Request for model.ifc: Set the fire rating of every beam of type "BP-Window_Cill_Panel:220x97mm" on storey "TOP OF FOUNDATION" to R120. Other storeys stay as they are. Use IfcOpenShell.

First a look at what the model holds.

```python
import ifcopenshell
import ifcopenshell.util.element

model = ifcopenshell.open("model.ifc")
print(model.schema)
storey = next(s for s in model.by_type("IfcBuildingStorey") if s.Name == "TOP OF FOUNDATION")
beams = [e for e in ifcopenshell.util.element.get_decomposition(storey) if e.is_a("IfcBeam")]
seen = {}
for e in beams:
    element_type = ifcopenshell.util.element.get_type(e)
    key = (element_type.Name if element_type != e and element_type else None, ifcopenshell.util.element.get_pset(e, "Pset_BeamCommon", "FireRating"))
    seen[key] = seen.get(key, 0) + 1
for (name, value), count in sorted(seen.items(), key=str):
    print(count, "x", name, "|", value)
```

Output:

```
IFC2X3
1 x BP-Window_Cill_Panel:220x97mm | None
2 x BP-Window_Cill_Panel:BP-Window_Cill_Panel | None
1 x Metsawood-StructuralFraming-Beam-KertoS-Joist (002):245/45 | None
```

```python
import ifcopenshell
import ifcopenshell.api.pset
import ifcopenshell.util.element

model = ifcopenshell.open("model.ifc")

storey = next(s for s in model.by_type("IfcBuildingStorey") if s.Name == "TOP OF FOUNDATION")
beams = [e for e in ifcopenshell.util.element.get_decomposition(storey) if e.is_a("IfcBeam")]

count = 0
for e in beams:
    element_type = ifcopenshell.util.element.get_type(e)
    if element_type in (None, e) or element_type.Name != "BP-Window_Cill_Panel:220x97mm":
        continue
    # add_pset returns the element's existing set when there is one.
    pset = ifcopenshell.api.pset.add_pset(model, product=e, name="Pset_BeamCommon")
    ifcopenshell.api.pset.edit_pset(model, pset=pset, properties={"FireRating": "R120"})
    count += 1

print(count, "beams updated")

model.write("model_v2.ifc")
```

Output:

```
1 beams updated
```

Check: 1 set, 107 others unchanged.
